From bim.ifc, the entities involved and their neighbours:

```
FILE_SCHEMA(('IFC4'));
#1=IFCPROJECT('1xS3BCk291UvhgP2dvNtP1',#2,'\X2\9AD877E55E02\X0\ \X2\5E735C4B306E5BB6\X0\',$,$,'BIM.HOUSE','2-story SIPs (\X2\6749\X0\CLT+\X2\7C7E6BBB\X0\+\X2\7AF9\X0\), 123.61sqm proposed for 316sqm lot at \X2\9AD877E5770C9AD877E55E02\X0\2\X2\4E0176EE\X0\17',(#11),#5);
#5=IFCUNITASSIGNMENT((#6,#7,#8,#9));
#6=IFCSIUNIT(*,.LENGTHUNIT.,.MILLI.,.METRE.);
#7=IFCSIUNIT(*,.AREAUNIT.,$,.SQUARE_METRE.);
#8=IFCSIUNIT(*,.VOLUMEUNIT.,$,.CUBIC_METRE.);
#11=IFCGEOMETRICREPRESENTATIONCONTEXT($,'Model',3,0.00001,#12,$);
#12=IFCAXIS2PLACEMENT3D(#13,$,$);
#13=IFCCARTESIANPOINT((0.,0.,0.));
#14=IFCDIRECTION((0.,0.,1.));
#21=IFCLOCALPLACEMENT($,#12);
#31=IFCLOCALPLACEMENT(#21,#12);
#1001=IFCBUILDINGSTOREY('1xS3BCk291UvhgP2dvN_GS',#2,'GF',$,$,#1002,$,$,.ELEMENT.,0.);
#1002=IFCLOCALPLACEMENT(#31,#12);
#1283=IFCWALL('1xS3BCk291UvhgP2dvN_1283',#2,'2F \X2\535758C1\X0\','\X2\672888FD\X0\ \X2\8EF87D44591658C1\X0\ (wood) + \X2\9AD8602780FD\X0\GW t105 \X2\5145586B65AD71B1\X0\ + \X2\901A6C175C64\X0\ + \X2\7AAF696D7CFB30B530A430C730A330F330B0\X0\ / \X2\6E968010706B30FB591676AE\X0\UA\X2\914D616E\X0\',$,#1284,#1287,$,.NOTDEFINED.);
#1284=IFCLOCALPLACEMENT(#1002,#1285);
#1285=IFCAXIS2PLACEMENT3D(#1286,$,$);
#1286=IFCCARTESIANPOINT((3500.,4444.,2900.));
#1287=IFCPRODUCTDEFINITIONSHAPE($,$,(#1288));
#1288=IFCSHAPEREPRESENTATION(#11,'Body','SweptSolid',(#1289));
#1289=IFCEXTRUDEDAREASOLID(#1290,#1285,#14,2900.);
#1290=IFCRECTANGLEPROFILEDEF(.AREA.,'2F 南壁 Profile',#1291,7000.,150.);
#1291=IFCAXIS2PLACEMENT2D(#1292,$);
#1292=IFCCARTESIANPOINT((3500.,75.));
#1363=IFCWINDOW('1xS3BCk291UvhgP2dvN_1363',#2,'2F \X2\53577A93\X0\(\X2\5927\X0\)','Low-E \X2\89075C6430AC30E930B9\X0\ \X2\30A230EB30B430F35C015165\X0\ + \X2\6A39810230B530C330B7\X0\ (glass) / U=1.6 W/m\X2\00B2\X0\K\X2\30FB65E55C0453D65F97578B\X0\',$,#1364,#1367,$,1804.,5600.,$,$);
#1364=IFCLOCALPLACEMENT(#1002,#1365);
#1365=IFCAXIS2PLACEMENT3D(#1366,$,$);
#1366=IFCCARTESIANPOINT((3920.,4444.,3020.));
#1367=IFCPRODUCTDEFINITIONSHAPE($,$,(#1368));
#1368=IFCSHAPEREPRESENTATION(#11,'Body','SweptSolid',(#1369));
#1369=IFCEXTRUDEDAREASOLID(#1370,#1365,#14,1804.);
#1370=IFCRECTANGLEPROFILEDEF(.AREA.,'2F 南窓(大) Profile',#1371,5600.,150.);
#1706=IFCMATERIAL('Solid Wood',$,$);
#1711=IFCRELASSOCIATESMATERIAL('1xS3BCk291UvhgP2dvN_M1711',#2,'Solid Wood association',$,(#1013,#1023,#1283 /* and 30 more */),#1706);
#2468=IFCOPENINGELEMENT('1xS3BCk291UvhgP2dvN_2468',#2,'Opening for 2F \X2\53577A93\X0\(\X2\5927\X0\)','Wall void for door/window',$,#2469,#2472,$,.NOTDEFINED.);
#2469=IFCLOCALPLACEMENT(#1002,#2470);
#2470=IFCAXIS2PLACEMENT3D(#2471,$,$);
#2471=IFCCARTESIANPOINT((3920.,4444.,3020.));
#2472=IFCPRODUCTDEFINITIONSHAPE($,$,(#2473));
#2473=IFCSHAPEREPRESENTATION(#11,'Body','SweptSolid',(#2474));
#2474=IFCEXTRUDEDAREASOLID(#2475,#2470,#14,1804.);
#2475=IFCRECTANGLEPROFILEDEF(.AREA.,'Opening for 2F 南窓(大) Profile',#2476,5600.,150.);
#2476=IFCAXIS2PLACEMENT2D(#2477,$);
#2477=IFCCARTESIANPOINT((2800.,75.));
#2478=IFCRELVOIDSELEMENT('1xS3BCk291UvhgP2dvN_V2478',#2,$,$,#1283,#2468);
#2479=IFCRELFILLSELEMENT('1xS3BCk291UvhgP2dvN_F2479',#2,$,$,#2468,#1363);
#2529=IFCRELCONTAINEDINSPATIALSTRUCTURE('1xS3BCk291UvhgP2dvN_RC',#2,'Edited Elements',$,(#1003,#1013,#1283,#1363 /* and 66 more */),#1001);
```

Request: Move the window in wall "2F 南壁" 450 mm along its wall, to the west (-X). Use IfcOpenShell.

```python
import ifcopenshell
import ifcopenshell.api.geometry
import ifcopenshell.util.placement
import ifcopenshell.util.unit

model = ifcopenshell.open("bim.ifc")
unit_scale = ifcopenshell.util.unit.calculate_unit_scale(model)

window = model.by_guid("1xS3BCk291UvhgP2dvN_1363")
opening = window.FillsVoids[0].RelatingOpeningElement
wall = opening.VoidsElements[0].RelatingBuildingElement

wall_matrix = ifcopenshell.util.placement.get_local_placement(wall.ObjectPlacement)
shift = wall_matrix[:3, 0] * -0.45 / unit_scale
before = ifcopenshell.util.placement.get_local_placement(window.ObjectPlacement)[:3, 3].copy()

# The window is not placed relative to its opening, so move both.
for product in (opening, window):
    matrix = ifcopenshell.util.placement.get_local_placement(product.ObjectPlacement)
    matrix[:3, 3] += shift
    ifcopenshell.api.geometry.edit_object_placement(model, product=product, matrix=matrix, is_si=False)

after = ifcopenshell.util.placement.get_local_placement(window.ObjectPlacement)[:3, 3]
print("window moved by", (after - before).round(3) + 0.0)

model.write("bim_updated.ifc")
```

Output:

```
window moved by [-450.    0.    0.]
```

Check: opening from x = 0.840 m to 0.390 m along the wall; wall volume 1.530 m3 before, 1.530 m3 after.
